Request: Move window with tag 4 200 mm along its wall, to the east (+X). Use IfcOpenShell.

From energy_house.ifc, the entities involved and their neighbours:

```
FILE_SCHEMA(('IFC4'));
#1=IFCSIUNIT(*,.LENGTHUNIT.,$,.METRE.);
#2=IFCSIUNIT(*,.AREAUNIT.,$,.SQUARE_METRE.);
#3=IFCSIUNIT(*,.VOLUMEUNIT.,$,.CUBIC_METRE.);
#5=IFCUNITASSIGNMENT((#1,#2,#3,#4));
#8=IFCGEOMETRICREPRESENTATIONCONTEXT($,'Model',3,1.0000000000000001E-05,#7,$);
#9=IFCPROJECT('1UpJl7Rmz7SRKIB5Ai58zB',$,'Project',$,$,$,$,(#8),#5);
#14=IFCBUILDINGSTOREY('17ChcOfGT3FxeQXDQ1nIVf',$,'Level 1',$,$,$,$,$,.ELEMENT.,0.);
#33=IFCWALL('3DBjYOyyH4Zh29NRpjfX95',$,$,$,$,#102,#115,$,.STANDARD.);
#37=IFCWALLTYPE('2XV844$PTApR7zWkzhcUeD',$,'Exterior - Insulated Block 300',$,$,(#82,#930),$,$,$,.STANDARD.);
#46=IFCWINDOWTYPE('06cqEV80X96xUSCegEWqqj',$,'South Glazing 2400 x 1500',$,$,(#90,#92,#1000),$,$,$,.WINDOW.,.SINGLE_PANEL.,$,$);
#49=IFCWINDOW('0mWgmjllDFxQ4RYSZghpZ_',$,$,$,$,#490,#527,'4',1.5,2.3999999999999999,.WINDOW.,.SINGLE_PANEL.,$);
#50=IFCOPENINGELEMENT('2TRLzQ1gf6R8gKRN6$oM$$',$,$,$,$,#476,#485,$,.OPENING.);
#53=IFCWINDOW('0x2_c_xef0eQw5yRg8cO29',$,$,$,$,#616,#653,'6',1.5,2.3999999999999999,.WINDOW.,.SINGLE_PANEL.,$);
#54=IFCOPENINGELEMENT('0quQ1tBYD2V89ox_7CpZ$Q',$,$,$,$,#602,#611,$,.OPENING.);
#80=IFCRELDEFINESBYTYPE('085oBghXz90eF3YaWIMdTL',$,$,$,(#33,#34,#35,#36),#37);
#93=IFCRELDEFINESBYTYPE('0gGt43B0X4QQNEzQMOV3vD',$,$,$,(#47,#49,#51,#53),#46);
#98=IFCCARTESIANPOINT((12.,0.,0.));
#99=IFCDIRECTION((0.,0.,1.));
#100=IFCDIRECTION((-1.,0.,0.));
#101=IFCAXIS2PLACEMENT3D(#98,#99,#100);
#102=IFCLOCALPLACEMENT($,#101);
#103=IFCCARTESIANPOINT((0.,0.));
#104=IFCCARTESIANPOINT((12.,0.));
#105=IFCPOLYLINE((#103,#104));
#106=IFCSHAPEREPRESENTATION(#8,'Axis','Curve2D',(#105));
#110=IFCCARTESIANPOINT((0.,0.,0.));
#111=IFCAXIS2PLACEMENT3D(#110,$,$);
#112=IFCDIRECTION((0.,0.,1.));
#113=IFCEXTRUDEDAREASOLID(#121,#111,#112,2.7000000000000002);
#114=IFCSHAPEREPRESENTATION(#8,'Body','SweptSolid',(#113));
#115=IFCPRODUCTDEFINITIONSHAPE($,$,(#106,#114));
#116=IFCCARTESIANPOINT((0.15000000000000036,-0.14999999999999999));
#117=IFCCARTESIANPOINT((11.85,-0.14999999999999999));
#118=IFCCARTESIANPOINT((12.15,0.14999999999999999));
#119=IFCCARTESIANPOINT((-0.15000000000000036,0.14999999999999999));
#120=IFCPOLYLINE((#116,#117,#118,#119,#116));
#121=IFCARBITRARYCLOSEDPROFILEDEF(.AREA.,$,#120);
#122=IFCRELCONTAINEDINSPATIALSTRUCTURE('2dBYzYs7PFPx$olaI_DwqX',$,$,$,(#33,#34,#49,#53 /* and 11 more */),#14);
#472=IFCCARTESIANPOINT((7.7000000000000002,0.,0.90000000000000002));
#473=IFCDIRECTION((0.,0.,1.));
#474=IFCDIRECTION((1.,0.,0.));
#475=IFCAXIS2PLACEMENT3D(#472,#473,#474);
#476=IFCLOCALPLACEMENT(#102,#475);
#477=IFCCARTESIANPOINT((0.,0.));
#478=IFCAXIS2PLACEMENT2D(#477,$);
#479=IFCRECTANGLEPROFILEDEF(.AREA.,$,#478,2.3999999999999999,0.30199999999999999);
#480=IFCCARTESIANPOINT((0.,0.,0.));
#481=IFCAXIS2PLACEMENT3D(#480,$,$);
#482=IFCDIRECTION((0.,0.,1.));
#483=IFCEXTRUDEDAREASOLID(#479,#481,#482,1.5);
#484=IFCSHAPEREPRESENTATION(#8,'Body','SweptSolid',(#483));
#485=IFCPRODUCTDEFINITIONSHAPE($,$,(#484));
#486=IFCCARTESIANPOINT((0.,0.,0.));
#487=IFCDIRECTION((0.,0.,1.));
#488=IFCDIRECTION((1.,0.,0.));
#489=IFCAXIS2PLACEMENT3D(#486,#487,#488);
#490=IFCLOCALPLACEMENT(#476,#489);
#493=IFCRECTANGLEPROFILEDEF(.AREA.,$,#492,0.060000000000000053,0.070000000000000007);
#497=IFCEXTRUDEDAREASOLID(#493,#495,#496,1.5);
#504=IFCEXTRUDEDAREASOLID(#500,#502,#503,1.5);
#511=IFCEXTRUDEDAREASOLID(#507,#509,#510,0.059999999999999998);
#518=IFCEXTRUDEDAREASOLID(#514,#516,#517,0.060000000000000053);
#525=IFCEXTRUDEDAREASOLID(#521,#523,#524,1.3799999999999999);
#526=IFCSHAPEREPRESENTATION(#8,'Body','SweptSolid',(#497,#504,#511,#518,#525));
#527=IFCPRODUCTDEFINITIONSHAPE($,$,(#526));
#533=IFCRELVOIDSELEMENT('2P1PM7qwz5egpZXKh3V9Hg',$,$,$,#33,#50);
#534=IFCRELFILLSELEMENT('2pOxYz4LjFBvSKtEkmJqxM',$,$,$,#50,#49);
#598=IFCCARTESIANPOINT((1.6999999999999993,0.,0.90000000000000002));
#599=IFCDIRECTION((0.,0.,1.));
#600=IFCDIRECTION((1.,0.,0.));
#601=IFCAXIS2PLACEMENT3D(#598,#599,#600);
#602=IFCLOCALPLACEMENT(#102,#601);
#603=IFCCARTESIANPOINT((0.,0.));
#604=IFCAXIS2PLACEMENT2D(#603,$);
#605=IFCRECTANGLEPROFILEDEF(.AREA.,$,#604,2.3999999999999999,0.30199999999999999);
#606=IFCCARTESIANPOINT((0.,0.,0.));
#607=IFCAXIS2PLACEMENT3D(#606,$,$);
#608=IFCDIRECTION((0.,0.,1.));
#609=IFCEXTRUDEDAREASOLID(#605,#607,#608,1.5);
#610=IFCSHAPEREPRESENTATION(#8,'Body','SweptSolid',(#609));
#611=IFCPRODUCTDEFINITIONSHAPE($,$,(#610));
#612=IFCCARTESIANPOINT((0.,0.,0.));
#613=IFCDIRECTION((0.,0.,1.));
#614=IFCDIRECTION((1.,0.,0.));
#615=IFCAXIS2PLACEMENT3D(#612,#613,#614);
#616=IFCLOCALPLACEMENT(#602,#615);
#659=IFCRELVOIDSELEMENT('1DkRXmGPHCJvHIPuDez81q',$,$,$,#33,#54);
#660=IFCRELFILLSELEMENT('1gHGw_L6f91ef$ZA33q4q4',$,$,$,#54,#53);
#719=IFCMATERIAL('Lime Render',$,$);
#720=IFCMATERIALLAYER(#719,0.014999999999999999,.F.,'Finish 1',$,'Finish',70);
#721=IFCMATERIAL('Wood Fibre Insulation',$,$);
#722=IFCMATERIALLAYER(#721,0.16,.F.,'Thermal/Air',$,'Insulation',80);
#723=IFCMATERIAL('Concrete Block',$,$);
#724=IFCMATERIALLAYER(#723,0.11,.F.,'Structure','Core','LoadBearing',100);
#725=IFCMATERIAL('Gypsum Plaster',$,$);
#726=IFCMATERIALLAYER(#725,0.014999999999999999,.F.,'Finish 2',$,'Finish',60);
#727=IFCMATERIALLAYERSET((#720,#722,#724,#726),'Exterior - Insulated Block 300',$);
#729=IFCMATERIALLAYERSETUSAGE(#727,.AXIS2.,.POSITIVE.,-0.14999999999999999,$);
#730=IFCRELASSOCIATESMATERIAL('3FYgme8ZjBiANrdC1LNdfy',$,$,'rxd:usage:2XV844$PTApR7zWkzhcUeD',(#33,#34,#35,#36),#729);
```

```python
import ifcopenshell
import ifcopenshell.api.geometry
import ifcopenshell.util.placement

model = ifcopenshell.open("energy_house.ifc")

window = model.by_id(49)
opening = window.FillsVoids[0].RelatingOpeningElement
wall = opening.VoidsElements[0].RelatingBuildingElement

wall_matrix = ifcopenshell.util.placement.get_local_placement(wall.ObjectPlacement)
shift = wall_matrix[:3, 0] * -0.2
before = ifcopenshell.util.placement.get_local_placement(window.ObjectPlacement)[:3, 3].copy()

# The window is placed relative to its opening, so it follows when the opening moves.
matrix = ifcopenshell.util.placement.get_local_placement(opening.ObjectPlacement)
matrix[:3, 3] += shift
ifcopenshell.api.geometry.edit_object_placement(
    model, product=opening, matrix=matrix, is_si=False, should_transform_children=True
)

after = ifcopenshell.util.placement.get_local_placement(window.ObjectPlacement)[:3, 3]
print("window moved by", (after - before).round(3) + 0.0)

model.write("energy_house_edited.ifc")
```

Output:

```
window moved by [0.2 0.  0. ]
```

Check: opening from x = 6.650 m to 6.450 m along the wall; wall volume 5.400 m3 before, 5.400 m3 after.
